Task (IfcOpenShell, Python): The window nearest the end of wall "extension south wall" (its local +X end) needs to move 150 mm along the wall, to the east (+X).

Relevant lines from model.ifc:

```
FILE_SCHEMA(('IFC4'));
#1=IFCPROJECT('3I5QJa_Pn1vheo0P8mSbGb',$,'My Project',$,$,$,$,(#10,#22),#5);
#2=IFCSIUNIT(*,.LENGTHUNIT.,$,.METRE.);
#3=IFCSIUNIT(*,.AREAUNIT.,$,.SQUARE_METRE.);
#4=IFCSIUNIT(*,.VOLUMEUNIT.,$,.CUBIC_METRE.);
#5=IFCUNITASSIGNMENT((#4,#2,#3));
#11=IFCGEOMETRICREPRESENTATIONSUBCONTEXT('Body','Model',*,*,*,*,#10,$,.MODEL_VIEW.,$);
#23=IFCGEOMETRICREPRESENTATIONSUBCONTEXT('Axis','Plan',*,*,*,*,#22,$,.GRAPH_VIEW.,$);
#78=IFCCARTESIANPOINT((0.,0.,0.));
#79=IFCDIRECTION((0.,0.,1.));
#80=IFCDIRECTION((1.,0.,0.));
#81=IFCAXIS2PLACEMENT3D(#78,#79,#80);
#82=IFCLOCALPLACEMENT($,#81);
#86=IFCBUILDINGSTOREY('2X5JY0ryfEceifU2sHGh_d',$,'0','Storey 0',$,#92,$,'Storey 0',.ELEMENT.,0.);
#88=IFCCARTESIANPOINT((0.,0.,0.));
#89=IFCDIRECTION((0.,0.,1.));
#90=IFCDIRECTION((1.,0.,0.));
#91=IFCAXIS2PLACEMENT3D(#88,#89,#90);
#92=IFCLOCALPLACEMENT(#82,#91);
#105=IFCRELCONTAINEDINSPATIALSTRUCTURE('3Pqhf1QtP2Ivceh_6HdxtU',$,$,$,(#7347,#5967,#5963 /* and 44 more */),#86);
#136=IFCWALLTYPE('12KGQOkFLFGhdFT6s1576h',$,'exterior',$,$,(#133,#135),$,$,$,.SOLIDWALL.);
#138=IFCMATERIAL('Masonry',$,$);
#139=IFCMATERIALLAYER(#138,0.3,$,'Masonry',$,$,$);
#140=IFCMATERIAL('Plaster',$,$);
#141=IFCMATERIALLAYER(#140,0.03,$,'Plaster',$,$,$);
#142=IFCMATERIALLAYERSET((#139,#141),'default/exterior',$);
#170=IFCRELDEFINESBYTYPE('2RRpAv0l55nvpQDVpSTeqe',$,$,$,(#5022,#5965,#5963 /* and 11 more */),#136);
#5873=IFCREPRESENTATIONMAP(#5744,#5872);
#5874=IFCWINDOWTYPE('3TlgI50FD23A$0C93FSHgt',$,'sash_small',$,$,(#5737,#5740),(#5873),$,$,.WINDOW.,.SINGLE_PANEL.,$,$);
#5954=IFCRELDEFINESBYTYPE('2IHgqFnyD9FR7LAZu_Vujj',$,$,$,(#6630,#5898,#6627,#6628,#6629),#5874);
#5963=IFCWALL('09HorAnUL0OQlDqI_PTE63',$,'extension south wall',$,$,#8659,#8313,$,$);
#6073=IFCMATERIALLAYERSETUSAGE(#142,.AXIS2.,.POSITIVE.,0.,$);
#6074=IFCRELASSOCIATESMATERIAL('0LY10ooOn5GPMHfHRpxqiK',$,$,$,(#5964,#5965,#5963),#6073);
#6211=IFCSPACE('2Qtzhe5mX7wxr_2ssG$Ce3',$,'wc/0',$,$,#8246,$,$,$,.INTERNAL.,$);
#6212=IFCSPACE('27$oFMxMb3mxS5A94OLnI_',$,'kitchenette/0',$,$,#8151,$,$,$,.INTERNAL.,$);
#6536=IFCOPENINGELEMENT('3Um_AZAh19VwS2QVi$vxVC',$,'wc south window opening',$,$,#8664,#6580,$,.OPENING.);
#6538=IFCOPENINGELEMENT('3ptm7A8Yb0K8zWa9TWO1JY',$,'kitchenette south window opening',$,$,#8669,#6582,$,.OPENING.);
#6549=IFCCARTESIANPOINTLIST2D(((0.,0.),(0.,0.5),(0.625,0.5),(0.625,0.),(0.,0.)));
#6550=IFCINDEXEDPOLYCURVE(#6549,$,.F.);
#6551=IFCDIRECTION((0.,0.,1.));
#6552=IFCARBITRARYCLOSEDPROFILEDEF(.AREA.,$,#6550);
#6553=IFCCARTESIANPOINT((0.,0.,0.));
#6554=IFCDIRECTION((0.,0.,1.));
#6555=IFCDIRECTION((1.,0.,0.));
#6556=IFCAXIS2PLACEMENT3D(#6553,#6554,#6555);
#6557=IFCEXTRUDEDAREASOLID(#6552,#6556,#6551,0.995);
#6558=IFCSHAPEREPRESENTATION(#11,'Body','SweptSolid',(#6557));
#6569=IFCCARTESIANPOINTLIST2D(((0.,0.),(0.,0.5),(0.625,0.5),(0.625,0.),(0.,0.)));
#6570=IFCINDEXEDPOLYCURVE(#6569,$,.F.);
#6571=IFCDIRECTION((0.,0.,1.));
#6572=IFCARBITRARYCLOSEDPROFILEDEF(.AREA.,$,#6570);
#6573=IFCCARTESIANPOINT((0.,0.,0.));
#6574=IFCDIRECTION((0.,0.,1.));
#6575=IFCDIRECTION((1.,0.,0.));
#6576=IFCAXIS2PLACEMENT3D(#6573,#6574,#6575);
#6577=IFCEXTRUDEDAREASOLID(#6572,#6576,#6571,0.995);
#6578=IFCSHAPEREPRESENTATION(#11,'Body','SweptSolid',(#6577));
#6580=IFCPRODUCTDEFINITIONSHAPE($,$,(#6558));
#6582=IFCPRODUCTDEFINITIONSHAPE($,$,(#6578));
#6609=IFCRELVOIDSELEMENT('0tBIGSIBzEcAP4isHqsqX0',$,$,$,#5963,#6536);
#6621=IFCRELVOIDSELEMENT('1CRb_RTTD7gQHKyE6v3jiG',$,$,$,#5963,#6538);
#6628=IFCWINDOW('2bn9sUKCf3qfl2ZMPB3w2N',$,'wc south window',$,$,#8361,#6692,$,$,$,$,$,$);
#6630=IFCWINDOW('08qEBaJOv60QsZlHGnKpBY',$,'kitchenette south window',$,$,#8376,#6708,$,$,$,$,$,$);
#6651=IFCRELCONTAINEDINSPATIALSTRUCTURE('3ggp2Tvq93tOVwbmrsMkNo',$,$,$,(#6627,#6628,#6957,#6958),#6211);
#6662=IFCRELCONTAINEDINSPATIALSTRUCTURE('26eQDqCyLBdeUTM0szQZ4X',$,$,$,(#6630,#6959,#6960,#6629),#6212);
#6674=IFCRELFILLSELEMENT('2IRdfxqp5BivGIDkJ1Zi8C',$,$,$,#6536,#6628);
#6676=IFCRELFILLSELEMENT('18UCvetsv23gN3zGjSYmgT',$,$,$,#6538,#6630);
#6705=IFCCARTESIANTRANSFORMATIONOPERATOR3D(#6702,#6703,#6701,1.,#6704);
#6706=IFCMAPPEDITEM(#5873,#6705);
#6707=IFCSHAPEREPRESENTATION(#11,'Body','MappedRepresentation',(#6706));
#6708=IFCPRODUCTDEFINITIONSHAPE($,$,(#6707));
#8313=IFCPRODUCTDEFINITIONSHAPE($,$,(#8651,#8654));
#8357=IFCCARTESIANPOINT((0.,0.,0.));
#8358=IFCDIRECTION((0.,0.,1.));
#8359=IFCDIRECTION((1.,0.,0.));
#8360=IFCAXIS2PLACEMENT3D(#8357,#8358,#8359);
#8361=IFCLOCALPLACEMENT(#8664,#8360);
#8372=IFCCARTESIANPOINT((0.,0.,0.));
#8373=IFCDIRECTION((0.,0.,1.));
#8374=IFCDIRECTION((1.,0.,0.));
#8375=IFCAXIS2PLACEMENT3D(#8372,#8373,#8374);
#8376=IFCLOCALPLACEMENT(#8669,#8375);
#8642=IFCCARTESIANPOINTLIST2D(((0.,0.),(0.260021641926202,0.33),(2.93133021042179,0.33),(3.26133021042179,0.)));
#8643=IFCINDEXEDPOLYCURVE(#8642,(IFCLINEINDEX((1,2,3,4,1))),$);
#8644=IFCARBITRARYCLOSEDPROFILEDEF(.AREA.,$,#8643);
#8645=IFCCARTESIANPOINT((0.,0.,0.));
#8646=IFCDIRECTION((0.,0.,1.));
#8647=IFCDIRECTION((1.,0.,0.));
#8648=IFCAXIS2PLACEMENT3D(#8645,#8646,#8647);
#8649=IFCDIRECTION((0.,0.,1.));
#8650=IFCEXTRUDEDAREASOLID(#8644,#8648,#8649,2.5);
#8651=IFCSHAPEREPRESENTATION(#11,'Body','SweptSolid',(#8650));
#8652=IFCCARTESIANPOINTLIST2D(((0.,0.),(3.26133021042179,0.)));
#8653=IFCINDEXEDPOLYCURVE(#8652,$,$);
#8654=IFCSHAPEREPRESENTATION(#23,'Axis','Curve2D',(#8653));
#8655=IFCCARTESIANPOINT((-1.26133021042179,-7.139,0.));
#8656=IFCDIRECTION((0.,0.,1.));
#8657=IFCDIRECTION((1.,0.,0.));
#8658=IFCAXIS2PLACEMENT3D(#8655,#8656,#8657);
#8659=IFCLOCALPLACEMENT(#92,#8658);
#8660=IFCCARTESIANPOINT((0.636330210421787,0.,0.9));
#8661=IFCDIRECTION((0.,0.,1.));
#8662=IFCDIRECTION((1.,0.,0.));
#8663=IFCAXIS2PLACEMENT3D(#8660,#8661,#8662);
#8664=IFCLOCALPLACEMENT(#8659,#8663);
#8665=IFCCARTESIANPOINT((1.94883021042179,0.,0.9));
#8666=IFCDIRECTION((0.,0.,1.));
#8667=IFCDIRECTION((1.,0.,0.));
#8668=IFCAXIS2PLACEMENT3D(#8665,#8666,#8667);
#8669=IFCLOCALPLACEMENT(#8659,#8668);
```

```python
import ifcopenshell
import ifcopenshell.api.geometry
import ifcopenshell.util.placement

model = ifcopenshell.open("model.ifc")

window = model.by_guid("08qEBaJOv60QsZlHGnKpBY")
opening = window.FillsVoids[0].RelatingOpeningElement
wall = opening.VoidsElements[0].RelatingBuildingElement

wall_matrix = ifcopenshell.util.placement.get_local_placement(wall.ObjectPlacement)
shift = wall_matrix[:3, 0] * 0.15
before = ifcopenshell.util.placement.get_local_placement(window.ObjectPlacement)[:3, 3].copy()

# The window is placed relative to its opening, so it follows when the opening moves.
matrix = ifcopenshell.util.placement.get_local_placement(opening.ObjectPlacement)
matrix[:3, 3] += shift
ifcopenshell.api.geometry.edit_object_placement(
    model, product=opening, matrix=matrix, is_si=False, should_transform_children=True
)

after = ifcopenshell.util.placement.get_local_placement(window.ObjectPlacement)[:3, 3]
print("window moved by", (after - before).round(3) + 0.0)

model.write("model_rev.ifc")
```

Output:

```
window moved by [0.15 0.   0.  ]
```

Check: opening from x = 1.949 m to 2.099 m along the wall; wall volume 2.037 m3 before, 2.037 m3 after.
